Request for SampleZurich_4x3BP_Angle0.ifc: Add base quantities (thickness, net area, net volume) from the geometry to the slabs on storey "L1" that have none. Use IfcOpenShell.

First a look at what the model holds.

```python
import ifcopenshell
import ifcopenshell.util.element
import ifcopenshell.util.unit

model = ifcopenshell.open("SampleZurich_4x3BP_Angle0.ifc")
print(model.schema)
for unit_type in ("LENGTHUNIT", "AREAUNIT", "VOLUMEUNIT"):
    print(unit_type, ifcopenshell.util.unit.calculate_unit_scale(model, unit_type))
storey = next(s for s in model.by_type("IfcBuildingStorey") if s.Name == "L1")
slabs = [e for e in ifcopenshell.util.element.get_decomposition(storey) if e.is_a("IfcSlab")]
for e in sorted(slabs, key=lambda e: e.id()):
    print(e.id(), e.is_a(), e.Name, list(ifcopenshell.util.element.get_psets(e, qtos_only=True)), sep=" | ")
```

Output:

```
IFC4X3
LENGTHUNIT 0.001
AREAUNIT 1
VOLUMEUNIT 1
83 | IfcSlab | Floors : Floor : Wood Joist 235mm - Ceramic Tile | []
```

```python
import ifcopenshell
import ifcopenshell.api.pset
import ifcopenshell.geom
import ifcopenshell.util.element
import ifcopenshell.util.shape
import ifcopenshell.util.unit

model = ifcopenshell.open("SampleZurich_4x3BP_Angle0.ifc")
unit_scale = ifcopenshell.util.unit.calculate_unit_scale(model)
area_scale = ifcopenshell.util.unit.calculate_unit_scale(model, "AREAUNIT")
volume_scale = ifcopenshell.util.unit.calculate_unit_scale(model, "VOLUMEUNIT")
settings = ifcopenshell.geom.settings()

storey = next(s for s in model.by_type("IfcBuildingStorey") if s.Name == "L1")
slabs = [e for e in ifcopenshell.util.element.get_decomposition(storey) if e.is_a("IfcSlab")]

for e in sorted(slabs, key=lambda e: e.id()):
    if ifcopenshell.util.element.get_psets(e, qtos_only=True, should_inherit=False):
        continue
    # Geometry comes back in metres, in the element's own axes.
    shape = ifcopenshell.geom.create_shape(settings, e)
    values = {
        "Width": ifcopenshell.util.shape.get_z(shape.geometry) / unit_scale,
        "NetArea": ifcopenshell.util.shape.get_footprint_area(shape.geometry) / area_scale,
        "NetVolume": ifcopenshell.util.shape.get_volume(shape.geometry) / volume_scale,
    }
    qto = ifcopenshell.api.pset.add_qto(model, product=e, name="Qto_SlabBaseQuantities")
    ifcopenshell.api.pset.edit_qto(model, qto=qto, properties=values)
    print(e.id(), {k: round(v, 3) for k, v in values.items()})

model.write("SampleZurich_4x3BP_Angle0-out.ifc")
```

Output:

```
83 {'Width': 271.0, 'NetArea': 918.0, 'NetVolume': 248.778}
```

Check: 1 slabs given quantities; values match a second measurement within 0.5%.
